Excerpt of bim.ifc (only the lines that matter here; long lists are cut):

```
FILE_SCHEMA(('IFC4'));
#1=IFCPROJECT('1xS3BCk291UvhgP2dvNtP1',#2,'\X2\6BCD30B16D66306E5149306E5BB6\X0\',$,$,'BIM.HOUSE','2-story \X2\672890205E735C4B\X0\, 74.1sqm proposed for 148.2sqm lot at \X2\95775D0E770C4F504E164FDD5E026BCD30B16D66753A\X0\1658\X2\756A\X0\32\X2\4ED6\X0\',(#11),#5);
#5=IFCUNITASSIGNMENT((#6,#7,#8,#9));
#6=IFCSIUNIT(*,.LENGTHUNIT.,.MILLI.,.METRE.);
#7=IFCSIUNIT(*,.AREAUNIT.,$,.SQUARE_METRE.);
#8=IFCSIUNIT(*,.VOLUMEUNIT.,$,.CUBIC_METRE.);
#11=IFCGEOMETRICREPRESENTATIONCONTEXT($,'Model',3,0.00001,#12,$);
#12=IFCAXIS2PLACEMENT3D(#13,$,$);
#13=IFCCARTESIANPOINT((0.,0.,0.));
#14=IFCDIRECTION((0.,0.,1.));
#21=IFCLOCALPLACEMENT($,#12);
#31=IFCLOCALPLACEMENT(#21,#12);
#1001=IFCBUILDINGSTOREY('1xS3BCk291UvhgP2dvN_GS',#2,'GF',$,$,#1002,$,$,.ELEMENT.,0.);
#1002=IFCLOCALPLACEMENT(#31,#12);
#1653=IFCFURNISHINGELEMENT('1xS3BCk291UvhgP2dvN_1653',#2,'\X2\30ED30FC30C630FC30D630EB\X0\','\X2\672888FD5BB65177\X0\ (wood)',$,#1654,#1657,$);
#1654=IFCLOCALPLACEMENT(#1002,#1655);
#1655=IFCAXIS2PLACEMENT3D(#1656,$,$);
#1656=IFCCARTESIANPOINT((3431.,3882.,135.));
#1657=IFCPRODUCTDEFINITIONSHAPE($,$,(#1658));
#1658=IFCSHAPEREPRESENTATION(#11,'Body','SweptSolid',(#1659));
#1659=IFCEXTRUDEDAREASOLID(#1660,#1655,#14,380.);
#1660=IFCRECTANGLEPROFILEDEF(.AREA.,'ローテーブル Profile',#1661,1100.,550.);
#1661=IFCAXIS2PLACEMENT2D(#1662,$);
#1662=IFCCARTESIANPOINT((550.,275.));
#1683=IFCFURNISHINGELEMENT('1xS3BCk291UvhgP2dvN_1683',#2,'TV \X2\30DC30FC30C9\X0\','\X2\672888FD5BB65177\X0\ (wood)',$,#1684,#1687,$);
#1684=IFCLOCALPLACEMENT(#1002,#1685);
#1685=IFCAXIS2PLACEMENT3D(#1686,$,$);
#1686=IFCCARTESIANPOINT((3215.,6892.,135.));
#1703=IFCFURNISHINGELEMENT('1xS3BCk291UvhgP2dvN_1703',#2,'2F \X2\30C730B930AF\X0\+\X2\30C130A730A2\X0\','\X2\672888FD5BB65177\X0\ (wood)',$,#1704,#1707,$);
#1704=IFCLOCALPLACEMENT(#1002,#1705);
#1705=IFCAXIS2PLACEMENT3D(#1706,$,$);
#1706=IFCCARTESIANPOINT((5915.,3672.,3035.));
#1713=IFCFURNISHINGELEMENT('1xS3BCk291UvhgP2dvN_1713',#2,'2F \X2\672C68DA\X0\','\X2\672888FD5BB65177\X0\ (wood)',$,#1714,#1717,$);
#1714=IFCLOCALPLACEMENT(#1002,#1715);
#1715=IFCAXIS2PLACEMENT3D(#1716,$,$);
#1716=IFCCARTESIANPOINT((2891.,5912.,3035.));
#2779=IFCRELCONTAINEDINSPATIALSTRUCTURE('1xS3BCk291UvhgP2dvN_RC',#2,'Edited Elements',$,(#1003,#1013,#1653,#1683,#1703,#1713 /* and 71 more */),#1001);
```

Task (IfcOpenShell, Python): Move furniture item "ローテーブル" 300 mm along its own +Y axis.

```python
import ifcopenshell
import ifcopenshell.api.geometry
import ifcopenshell.util.placement
import ifcopenshell.util.unit

model = ifcopenshell.open("bim.ifc")
unit_scale = ifcopenshell.util.unit.calculate_unit_scale(model)

item = model.by_id(1653)
matrix = ifcopenshell.util.placement.get_local_placement(item.ObjectPlacement)
matrix[:3, 3] += matrix[:3, 1] * 0.3 / unit_scale
ifcopenshell.api.geometry.edit_object_placement(model, product=item, matrix=matrix, is_si=False)

print(ifcopenshell.util.placement.get_local_placement(item.ObjectPlacement).round(3) + 0.0)

model.write("bim_rev.ifc")
```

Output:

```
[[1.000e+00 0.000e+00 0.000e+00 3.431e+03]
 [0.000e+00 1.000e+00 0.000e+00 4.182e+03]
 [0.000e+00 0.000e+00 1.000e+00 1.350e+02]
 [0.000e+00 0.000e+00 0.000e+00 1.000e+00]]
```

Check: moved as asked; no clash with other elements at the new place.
